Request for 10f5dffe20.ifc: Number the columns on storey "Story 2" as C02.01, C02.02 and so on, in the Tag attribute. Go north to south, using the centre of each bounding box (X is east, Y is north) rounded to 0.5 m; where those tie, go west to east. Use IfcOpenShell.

First a look at what the model holds.

```python
import ifcopenshell
import ifcopenshell.util.element
import ifcopenshell.util.placement

model = ifcopenshell.open("10f5dffe20.ifc")
print(model.schema)
storey = next(s for s in model.by_type("IfcBuildingStorey") if s.Name == "Story 2")
columns = [e for e in ifcopenshell.util.element.get_decomposition(storey) if e.is_a("IfcColumn")]
for e in sorted(columns, key=lambda e: e.id()):
    origin = ifcopenshell.util.placement.get_local_placement(e.ObjectPlacement)[:3, 3]
    print(e.id(), e.Tag, e.Name, origin.round(2) + 0.0, sep=" | ")
```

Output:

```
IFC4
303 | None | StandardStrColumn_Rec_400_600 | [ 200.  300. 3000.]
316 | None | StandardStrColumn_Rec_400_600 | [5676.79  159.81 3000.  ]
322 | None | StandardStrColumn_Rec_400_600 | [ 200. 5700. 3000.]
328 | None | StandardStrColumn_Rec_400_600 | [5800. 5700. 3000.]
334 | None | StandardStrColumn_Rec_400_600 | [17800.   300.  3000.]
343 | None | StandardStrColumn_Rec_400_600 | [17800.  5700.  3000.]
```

```python
import ifcopenshell
import ifcopenshell.geom
import ifcopenshell.util.element
import ifcopenshell.util.shape

model = ifcopenshell.open("10f5dffe20.ifc")
settings = ifcopenshell.geom.settings()
settings.set("use-world-coords", True)


def centre(element):
    shape = ifcopenshell.geom.create_shape(settings, element)
    return ifcopenshell.util.shape.get_bbox_centroid(shape.geometry)


storey = next(s for s in model.by_type("IfcBuildingStorey") if s.Name == "Story 2")
columns = [e for e in ifcopenshell.util.element.get_decomposition(storey) if e.is_a("IfcColumn")]

# Insertion points can sit at a corner or the storey origin, so sort by the geometry (in metres).
centres = {e: centre(e) for e in columns}
columns.sort(key=lambda e: (-round(centres[e][1] / 0.5), centres[e][0]))

for i, e in enumerate(columns, start=1):
    number = f"C02.{i:02d}"
    e.Tag = number
    print(e.id(), number)

model.write("10f5dffe20_updated.ifc")
```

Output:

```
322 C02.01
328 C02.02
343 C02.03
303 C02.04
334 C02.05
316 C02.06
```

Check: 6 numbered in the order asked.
